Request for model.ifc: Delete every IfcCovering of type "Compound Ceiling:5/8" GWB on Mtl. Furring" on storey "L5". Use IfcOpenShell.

First a look at what the model holds.

```python
import ifcopenshell
import ifcopenshell.util.element

model = ifcopenshell.open("model.ifc")
print(model.schema)
storey = next(s for s in model.by_type("IfcBuildingStorey") if s.Name == "L5")
coverings = [e for e in ifcopenshell.util.element.get_decomposition(storey) if e.is_a("IfcCovering")]
seen = {}
for e in coverings:
    element_type = ifcopenshell.util.element.get_type(e)
    name = element_type.Name if element_type not in (None, e) else None
    seen[name] = seen.get(name, 0) + 1
for name, count in sorted(seen.items(), key=str):
    print(count, "x", name)
```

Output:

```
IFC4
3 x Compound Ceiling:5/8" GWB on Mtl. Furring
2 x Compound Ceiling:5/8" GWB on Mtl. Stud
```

```python
import ifcopenshell
import ifcopenshell.api.root
import ifcopenshell.util.element

model = ifcopenshell.open("model.ifc")

storey = next(s for s in model.by_type("IfcBuildingStorey") if s.Name == "L5")
coverings = [e for e in ifcopenshell.util.element.get_decomposition(storey) if e.is_a("IfcCovering")]
targets = [e for e in coverings if (t := ifcopenshell.util.element.get_type(e)) not in (None, e) and t.Name == 'Compound Ceiling:5/8" GWB on Mtl. Furring']

for e in targets:
    ifcopenshell.api.root.remove_product(model, product=e)
print(len(targets), "removed")

model.write("model_rev.ifc")
```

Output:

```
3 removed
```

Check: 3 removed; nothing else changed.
